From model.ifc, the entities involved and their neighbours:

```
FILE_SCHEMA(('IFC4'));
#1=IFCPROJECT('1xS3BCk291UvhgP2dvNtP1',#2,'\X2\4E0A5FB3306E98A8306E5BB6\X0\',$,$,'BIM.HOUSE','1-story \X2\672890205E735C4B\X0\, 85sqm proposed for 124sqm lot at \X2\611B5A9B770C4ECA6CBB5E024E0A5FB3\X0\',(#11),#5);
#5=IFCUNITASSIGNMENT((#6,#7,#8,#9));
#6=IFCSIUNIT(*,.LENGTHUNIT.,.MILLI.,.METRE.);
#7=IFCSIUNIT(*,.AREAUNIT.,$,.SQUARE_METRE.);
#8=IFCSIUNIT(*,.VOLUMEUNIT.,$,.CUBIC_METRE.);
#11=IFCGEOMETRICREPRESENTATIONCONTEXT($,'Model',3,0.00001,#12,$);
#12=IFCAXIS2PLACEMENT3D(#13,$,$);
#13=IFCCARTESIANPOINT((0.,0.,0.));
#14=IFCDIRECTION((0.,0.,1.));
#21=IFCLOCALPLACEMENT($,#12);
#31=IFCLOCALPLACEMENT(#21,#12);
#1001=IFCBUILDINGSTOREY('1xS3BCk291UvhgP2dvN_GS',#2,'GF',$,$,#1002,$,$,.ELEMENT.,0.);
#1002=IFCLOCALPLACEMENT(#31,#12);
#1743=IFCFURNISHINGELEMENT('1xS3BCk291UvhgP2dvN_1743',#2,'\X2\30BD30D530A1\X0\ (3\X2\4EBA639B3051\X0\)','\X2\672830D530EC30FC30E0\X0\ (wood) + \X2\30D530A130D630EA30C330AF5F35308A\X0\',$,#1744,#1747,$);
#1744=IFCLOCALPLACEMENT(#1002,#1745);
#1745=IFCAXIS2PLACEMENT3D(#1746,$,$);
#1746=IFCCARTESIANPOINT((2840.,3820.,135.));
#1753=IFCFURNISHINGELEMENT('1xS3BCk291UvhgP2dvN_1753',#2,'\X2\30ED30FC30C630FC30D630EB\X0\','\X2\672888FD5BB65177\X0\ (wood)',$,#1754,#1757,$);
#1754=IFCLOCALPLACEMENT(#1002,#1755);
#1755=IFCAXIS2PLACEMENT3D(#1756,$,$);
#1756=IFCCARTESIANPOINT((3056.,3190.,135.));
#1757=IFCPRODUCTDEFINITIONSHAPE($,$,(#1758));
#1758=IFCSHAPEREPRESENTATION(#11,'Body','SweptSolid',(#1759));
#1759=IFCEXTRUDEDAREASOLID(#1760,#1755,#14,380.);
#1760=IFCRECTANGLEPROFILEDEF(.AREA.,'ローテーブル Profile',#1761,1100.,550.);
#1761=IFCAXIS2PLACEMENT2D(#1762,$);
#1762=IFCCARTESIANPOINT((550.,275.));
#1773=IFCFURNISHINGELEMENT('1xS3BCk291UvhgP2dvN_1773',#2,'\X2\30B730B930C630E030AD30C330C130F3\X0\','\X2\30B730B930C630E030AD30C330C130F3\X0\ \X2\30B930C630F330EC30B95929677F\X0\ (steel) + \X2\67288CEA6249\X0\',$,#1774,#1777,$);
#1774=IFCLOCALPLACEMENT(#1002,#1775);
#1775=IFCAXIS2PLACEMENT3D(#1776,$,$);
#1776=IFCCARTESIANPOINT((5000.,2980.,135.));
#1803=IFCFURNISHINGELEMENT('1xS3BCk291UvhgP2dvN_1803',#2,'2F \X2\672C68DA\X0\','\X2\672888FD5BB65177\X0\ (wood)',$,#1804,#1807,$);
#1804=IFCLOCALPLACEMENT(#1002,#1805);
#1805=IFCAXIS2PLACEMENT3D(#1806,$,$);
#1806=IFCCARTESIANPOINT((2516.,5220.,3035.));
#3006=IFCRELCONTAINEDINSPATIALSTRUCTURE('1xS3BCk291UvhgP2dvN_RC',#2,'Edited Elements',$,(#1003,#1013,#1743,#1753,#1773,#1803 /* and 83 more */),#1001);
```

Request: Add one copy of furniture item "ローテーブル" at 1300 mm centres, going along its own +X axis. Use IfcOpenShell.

```python
import ifcopenshell
import ifcopenshell.api.geometry
import ifcopenshell.api.root
import ifcopenshell.util.element
import ifcopenshell.util.placement

model = ifcopenshell.open("model.ifc")


def reuse_history(source, copy):
    """copy_class also copies each property set's owner history, people and application; keep the originals."""
    for rel in copy.IsDefinedBy:
        if rel.is_a("IfcRelDefinesByProperties") and (history := rel.RelatingPropertyDefinition.OwnerHistory):
            rel.RelatingPropertyDefinition.OwnerHistory = source.OwnerHistory
            ifcopenshell.util.element.remove_deep2(model, history)


source = model.by_guid("1xS3BCk291UvhgP2dvN_1753")
base = ifcopenshell.util.placement.get_local_placement(source.ObjectPlacement)
step = base[:3, 0] * 1300.0

for i in range(1, 2):
    copy = ifcopenshell.api.root.copy_class(model, product=source)
    copy.Representation = ifcopenshell.util.element.copy_deep(
        model, source.Representation, exclude=["IfcGeometricRepresentationContext", "IfcRepresentationMap"]
    )
    reuse_history(source, copy)
    matrix = base.copy()
    matrix[:3, 3] += i * step
    print("added at", matrix[:3, 3].round(3) + 0.0)
    ifcopenshell.api.geometry.edit_object_placement(model, product=copy, matrix=matrix, is_si=False)

model.write("model_rev.ifc")
```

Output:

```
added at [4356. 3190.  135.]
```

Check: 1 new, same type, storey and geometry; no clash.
